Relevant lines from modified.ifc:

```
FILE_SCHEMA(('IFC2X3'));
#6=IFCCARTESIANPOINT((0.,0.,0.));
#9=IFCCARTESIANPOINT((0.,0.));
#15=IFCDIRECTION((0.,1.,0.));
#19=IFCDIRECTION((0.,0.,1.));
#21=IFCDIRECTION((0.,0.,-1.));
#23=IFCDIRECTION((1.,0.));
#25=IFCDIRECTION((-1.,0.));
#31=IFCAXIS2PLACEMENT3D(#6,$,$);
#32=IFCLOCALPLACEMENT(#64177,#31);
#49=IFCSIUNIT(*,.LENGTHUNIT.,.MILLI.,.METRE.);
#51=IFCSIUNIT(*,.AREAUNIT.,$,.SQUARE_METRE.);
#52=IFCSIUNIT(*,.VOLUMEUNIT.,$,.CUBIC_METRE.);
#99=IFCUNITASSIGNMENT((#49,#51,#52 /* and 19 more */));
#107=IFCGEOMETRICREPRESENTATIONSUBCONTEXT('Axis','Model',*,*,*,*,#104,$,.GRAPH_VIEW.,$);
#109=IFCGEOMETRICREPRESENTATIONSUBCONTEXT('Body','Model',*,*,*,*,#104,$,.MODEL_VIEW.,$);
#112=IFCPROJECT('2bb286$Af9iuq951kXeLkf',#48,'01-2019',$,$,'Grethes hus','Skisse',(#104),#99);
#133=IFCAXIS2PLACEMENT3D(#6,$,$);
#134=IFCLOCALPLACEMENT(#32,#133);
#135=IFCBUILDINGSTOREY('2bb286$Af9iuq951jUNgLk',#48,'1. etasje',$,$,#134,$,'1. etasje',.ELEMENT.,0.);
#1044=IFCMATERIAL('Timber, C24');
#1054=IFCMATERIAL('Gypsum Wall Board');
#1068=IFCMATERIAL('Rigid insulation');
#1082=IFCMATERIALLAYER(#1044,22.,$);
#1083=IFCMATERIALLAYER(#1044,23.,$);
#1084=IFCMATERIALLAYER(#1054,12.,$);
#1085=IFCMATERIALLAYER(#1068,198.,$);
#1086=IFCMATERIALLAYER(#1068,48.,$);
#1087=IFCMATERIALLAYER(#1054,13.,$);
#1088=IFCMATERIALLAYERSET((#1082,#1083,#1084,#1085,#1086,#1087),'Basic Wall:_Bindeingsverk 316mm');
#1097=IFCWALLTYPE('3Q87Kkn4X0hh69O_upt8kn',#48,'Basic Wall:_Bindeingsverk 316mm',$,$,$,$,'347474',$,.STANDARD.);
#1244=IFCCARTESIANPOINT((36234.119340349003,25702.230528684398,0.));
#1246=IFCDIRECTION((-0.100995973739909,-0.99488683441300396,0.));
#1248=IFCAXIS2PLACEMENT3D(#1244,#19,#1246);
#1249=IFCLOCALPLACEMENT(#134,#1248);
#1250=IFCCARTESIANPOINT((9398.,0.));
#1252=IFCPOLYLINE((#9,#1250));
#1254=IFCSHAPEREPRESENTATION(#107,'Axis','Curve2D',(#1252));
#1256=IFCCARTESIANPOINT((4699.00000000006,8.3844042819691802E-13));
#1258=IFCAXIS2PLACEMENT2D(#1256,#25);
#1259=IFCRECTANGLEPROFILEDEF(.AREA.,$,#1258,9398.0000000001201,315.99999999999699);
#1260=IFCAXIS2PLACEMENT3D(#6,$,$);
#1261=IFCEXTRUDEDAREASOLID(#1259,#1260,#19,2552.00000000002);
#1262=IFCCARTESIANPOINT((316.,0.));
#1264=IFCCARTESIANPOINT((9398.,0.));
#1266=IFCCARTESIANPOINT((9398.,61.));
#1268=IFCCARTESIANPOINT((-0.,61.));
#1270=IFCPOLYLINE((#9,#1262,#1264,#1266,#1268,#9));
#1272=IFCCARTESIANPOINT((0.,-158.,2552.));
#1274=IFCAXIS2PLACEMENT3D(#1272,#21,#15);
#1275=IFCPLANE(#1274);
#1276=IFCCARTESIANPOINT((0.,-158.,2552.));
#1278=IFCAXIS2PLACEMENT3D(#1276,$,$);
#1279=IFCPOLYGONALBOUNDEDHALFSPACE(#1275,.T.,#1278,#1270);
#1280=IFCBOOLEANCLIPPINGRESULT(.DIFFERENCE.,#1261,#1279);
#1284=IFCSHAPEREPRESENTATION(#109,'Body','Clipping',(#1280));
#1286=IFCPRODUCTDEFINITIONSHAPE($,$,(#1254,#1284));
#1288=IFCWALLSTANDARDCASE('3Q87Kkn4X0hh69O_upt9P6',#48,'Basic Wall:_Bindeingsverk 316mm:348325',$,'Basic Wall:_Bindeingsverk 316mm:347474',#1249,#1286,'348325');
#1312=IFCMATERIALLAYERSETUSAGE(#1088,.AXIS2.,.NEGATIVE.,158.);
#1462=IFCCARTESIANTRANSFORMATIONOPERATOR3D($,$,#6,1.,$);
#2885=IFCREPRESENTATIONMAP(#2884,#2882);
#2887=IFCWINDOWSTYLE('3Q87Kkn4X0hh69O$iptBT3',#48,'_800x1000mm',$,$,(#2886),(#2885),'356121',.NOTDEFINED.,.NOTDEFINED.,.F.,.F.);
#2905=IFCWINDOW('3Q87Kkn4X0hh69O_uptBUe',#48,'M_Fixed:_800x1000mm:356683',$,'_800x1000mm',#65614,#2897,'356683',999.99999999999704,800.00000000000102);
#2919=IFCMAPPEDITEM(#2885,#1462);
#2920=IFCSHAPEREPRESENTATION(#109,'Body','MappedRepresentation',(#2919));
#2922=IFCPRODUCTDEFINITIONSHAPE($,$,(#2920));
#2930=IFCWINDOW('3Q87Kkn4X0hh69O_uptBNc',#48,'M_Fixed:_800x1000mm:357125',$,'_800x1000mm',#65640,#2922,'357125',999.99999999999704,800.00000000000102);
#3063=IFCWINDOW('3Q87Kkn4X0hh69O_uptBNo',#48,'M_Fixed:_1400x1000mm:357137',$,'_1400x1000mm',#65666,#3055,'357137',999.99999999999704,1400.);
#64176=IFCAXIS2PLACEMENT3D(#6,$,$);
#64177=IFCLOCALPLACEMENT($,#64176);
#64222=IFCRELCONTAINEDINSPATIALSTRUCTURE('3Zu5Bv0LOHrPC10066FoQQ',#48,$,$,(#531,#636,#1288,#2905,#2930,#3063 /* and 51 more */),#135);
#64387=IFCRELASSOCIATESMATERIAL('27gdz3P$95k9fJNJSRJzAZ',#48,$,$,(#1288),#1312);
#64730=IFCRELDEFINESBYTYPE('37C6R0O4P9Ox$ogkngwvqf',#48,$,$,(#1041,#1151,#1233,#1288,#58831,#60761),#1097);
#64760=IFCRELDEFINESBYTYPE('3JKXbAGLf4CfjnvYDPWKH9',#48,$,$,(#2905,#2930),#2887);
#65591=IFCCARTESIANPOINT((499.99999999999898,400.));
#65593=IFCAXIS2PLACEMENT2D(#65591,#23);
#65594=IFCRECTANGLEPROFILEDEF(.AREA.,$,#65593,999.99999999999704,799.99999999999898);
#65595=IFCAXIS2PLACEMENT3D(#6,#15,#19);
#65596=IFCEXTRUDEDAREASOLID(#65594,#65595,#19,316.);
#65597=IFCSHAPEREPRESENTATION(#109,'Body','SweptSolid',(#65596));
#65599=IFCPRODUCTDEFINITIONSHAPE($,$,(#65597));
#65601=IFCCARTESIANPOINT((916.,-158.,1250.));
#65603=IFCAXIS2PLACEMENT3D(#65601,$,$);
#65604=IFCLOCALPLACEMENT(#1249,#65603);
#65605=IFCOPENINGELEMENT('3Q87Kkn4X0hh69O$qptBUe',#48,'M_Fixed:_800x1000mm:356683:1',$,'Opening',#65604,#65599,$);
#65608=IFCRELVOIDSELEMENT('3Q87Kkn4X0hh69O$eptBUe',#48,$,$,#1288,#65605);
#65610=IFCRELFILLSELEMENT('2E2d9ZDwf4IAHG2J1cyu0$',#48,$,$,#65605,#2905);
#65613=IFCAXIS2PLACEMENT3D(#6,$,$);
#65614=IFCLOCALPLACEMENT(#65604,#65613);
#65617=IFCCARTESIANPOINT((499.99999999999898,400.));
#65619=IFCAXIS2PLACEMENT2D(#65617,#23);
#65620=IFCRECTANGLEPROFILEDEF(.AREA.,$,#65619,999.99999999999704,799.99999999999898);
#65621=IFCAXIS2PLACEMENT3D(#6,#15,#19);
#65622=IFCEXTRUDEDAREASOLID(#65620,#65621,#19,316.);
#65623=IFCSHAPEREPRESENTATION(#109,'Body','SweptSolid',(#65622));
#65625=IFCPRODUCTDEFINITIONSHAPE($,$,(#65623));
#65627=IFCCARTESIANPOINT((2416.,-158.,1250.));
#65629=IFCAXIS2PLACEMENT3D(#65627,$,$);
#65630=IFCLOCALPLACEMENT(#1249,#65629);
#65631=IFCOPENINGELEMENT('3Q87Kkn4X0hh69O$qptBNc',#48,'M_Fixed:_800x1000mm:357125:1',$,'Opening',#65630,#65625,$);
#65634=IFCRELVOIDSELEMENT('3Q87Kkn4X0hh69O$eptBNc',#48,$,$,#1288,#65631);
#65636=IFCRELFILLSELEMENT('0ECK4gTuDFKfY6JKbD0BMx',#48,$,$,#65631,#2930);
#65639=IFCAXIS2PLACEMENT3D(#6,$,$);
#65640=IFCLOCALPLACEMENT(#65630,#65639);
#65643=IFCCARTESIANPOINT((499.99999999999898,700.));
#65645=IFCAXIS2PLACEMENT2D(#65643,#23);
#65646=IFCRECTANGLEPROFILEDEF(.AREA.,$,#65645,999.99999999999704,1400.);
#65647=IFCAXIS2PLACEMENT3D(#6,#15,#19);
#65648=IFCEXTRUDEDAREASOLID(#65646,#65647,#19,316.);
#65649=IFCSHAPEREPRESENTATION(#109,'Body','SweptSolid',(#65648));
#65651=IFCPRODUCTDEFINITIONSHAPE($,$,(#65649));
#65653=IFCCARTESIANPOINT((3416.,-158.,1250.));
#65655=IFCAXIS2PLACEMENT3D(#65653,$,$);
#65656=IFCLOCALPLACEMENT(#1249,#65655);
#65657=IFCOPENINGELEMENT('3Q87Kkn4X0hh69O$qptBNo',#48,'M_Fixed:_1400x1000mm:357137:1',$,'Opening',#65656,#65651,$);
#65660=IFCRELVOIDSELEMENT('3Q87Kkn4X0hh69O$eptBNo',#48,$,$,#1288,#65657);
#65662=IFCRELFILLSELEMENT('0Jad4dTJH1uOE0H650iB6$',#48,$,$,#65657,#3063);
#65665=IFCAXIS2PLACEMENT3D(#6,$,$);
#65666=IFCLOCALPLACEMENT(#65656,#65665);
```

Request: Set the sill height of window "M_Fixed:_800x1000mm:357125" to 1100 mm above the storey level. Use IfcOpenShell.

```python
import numpy as np
import ifcopenshell
import ifcopenshell.api.geometry
import ifcopenshell.geom
import ifcopenshell.util.element
import ifcopenshell.util.placement
import ifcopenshell.util.shape
import ifcopenshell.util.unit

model = ifcopenshell.open("modified.ifc")
unit_scale = ifcopenshell.util.unit.calculate_unit_scale(model)

window = model.by_guid("3Q87Kkn4X0hh69O_uptBNc")
opening = window.FillsVoids[0].RelatingOpeningElement
storey = ifcopenshell.util.element.get_container(window, ifc_class="IfcBuildingStorey")
level = ifcopenshell.util.placement.get_local_placement(storey.ObjectPlacement)[2, 3]

# The opening's origin need not be at the sill, so measure its lowest point.
shape = ifcopenshell.geom.create_shape(ifcopenshell.geom.settings(), opening)
bottom = ifcopenshell.util.shape.get_shape_bottom_elevation(shape, shape.geometry) / unit_scale
dz = level + 1100.0 - bottom

shift = np.array([0.0, 0.0, dz])
# The window is placed relative to its opening, so it follows when the opening moves.
matrix = ifcopenshell.util.placement.get_local_placement(opening.ObjectPlacement)
matrix[:3, 3] += shift
ifcopenshell.api.geometry.edit_object_placement(
    model, product=opening, matrix=matrix, is_si=False, should_transform_children=True
)

print(f"moved by {dz * unit_scale:+.3f} m")

model.write("modified_edited.ifc")
```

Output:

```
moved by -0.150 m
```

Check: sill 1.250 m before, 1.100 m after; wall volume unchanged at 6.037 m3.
